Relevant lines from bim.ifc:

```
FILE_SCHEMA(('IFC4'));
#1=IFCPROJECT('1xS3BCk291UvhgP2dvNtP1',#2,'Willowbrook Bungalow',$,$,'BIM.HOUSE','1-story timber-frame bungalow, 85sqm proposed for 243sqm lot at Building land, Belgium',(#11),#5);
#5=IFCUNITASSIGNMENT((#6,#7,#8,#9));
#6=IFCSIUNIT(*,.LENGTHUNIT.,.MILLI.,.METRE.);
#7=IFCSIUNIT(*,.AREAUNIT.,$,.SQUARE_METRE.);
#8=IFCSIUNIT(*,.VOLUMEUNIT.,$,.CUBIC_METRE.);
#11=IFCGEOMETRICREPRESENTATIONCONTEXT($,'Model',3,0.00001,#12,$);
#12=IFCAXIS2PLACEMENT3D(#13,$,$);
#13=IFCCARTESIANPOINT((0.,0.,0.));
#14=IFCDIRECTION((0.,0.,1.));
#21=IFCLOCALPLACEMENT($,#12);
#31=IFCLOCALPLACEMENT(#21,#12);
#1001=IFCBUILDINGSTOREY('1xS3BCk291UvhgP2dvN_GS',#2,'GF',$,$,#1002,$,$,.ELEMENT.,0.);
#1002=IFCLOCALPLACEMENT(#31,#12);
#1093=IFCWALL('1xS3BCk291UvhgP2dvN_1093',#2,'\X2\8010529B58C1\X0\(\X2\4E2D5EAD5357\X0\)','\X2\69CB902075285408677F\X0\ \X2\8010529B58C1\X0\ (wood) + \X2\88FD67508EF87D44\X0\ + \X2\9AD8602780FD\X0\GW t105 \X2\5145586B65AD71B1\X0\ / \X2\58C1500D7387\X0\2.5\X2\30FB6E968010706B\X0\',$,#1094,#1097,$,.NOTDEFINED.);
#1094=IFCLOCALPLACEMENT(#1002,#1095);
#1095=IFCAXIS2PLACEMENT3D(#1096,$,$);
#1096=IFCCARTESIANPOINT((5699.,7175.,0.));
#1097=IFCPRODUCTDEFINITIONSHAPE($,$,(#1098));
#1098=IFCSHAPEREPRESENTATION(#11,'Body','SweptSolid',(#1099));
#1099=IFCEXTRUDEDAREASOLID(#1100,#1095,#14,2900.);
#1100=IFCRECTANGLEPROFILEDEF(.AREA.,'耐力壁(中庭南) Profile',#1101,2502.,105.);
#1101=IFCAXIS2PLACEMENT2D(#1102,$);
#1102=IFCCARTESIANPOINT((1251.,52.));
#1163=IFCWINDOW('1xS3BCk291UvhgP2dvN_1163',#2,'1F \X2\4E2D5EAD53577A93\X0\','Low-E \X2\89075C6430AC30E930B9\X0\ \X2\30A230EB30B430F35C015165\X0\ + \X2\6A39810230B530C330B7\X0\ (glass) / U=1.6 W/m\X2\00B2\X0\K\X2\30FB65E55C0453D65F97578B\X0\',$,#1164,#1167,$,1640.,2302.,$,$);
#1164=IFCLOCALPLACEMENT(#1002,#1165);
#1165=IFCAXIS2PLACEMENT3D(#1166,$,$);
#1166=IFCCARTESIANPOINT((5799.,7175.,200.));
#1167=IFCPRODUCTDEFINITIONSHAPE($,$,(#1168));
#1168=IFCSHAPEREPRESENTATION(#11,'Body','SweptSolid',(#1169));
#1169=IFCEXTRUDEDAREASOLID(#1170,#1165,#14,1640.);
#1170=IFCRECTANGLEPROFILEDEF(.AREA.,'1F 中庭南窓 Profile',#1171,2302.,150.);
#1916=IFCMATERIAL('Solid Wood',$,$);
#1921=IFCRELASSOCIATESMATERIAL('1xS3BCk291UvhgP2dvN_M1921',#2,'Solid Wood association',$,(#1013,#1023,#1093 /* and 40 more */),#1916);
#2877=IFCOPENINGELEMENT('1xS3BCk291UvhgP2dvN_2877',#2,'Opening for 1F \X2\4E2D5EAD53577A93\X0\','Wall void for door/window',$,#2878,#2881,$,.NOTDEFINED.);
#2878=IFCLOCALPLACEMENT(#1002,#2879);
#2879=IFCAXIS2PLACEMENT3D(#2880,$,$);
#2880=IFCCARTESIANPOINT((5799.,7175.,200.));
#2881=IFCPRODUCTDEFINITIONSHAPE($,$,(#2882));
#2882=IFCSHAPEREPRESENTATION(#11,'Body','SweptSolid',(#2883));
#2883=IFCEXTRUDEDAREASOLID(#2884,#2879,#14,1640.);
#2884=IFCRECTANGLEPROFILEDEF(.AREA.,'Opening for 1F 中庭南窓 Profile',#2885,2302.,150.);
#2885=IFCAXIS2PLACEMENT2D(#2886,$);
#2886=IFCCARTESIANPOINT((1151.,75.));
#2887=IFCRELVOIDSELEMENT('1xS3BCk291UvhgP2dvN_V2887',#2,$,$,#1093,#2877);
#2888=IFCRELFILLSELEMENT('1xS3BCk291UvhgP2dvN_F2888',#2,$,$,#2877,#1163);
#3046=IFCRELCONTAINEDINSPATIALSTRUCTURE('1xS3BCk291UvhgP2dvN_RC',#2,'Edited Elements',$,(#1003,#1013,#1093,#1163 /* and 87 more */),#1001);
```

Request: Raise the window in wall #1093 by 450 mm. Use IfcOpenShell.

```python
import numpy as np
import ifcopenshell
import ifcopenshell.api.geometry
import ifcopenshell.util.placement
import ifcopenshell.util.unit

model = ifcopenshell.open("bim.ifc")
unit_scale = ifcopenshell.util.unit.calculate_unit_scale(model)

window = model.by_guid("1xS3BCk291UvhgP2dvN_1163")
opening = window.FillsVoids[0].RelatingOpeningElement
dz = 0.45 / unit_scale

shift = np.array([0.0, 0.0, dz])
# The window is not placed relative to its opening, so move both.
for product in (opening, window):
    matrix = ifcopenshell.util.placement.get_local_placement(product.ObjectPlacement)
    matrix[:3, 3] += shift
    ifcopenshell.api.geometry.edit_object_placement(model, product=product, matrix=matrix, is_si=False)

print(f"moved by {dz * unit_scale:+.3f} m")

model.write("bim_rev.ifc")
```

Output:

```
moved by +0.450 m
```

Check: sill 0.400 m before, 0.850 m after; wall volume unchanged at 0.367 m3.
